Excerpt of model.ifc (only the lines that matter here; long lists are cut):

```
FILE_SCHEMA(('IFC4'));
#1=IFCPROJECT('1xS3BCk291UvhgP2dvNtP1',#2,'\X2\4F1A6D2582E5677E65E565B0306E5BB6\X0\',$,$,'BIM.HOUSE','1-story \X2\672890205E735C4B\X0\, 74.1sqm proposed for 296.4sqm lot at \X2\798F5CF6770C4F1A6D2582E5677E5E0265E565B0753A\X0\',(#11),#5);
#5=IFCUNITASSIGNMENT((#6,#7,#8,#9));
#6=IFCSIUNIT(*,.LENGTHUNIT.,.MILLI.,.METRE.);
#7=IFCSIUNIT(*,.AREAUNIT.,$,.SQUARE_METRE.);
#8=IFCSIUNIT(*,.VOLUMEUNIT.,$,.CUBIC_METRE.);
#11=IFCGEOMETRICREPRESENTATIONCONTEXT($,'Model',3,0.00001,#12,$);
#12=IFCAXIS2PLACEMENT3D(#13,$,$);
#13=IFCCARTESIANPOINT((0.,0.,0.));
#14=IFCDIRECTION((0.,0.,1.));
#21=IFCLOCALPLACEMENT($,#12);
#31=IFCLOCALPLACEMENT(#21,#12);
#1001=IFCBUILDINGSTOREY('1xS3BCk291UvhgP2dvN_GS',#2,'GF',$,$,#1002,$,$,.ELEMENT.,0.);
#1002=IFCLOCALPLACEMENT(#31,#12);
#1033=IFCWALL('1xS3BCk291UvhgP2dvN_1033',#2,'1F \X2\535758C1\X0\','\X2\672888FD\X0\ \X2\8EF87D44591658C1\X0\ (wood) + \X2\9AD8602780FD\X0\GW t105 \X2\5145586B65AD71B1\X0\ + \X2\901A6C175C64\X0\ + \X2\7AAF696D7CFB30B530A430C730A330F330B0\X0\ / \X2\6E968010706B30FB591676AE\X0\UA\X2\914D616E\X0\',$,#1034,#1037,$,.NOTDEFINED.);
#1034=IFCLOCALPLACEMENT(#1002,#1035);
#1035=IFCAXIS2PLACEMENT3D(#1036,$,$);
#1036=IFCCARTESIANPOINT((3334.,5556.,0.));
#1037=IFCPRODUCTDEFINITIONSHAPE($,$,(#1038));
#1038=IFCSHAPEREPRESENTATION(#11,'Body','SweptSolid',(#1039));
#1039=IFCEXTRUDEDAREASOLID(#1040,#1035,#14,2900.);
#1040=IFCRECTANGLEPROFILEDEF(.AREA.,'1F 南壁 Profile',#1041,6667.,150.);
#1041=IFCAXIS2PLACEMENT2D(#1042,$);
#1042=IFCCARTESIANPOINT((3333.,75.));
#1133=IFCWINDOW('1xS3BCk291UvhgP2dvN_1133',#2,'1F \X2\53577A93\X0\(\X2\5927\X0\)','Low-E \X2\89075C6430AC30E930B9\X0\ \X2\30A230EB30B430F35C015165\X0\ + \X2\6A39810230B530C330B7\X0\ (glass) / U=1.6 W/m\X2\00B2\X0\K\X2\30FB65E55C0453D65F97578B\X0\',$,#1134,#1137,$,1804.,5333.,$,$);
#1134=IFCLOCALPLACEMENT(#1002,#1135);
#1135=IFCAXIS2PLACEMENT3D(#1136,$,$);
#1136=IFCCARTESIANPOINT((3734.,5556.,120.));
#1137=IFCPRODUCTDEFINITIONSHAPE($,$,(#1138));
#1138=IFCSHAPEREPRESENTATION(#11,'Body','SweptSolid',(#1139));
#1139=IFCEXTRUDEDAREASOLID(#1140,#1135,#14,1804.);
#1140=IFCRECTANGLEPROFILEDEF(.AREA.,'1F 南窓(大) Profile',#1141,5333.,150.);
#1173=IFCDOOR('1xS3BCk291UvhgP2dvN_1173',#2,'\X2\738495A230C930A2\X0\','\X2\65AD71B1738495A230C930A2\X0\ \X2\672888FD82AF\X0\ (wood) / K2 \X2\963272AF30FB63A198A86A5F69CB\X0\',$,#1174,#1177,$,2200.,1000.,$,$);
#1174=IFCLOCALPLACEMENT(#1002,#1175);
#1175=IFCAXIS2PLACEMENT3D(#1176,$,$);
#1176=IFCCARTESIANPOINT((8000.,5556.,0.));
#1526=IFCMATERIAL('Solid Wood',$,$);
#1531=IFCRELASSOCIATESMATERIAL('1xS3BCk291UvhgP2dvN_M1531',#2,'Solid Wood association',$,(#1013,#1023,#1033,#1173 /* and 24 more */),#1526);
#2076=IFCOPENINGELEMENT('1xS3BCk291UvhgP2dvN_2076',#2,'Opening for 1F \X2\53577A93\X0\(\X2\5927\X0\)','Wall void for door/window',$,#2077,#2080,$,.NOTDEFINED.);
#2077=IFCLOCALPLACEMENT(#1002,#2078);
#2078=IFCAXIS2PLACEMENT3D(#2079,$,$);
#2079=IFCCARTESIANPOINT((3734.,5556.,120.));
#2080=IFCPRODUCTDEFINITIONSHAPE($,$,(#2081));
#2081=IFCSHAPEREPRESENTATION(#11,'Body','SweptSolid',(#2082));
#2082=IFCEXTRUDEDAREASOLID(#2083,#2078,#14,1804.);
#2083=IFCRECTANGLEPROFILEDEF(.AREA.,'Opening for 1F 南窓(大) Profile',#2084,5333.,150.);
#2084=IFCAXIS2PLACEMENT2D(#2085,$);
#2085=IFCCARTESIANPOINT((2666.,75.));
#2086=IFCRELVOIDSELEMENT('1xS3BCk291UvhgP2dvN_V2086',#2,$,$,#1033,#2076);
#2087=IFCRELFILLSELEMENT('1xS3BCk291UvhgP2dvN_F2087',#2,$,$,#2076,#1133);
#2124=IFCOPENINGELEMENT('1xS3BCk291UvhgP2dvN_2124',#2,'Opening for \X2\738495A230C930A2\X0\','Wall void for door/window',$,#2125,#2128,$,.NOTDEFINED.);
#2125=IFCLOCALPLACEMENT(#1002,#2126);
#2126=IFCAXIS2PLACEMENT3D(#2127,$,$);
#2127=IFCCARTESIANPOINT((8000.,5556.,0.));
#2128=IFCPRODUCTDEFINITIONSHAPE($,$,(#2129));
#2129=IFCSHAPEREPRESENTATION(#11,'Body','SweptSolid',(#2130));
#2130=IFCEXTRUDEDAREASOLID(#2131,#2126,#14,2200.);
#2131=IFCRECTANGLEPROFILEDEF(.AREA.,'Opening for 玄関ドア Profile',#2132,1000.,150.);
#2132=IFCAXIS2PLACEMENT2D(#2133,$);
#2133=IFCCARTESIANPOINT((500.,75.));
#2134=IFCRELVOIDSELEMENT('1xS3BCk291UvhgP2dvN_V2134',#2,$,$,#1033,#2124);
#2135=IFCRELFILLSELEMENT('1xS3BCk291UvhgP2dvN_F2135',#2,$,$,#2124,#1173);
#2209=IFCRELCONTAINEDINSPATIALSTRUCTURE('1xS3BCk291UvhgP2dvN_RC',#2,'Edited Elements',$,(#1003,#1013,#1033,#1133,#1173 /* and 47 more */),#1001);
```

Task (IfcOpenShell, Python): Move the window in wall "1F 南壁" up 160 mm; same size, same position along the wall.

```python
import numpy as np
import ifcopenshell
import ifcopenshell.api.geometry
import ifcopenshell.util.placement
import ifcopenshell.util.unit

model = ifcopenshell.open("model.ifc")
unit_scale = ifcopenshell.util.unit.calculate_unit_scale(model)

window = model.by_guid("1xS3BCk291UvhgP2dvN_1133")
opening = window.FillsVoids[0].RelatingOpeningElement
dz = 160.0

shift = np.array([0.0, 0.0, dz])
# The window is not placed relative to its opening, so move both.
for product in (opening, window):
    matrix = ifcopenshell.util.placement.get_local_placement(product.ObjectPlacement)
    matrix[:3, 3] += shift
    ifcopenshell.api.geometry.edit_object_placement(model, product=product, matrix=matrix, is_si=False)

print(f"moved by {dz * unit_scale:+.3f} m")

model.write("model_rev.ifc")
```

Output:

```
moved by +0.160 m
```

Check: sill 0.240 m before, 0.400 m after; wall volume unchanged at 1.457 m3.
